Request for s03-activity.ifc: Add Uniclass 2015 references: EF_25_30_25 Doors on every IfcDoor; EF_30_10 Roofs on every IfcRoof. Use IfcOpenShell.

First a look at what the model holds.

```python
import ifcopenshell

model = ifcopenshell.open("s03-activity.ifc")
print(model.schema)
print("classifications:", [c.Name for c in model.by_type("IfcClassification")])
for ifc_class in ("IfcDoor", "IfcRoof", "IfcStair", "IfcWall", "IfcWindow"):
    print(ifc_class, len(model.by_type(ifc_class)))
```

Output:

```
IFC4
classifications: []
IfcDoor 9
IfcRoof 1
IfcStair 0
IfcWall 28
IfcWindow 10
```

```python
import ifcopenshell
import ifcopenshell.api.classification

model = ifcopenshell.open("s03-activity.ifc")

system = ifcopenshell.api.classification.add_classification(model, classification="Uniclass 2015")

codes = {
    "IfcDoor": ("EF_25_30_25", "Doors"),
    "IfcRoof": ("EF_30_10", "Roofs"),
}
for ifc_class, (code, name) in codes.items():
    products = model.by_type(ifc_class)
    ifcopenshell.api.classification.add_reference(
        model, products=products, classification=system, identification=code, name=name
    )
    print(code, len(products))

model.write("s03-activity_rev.ifc")
```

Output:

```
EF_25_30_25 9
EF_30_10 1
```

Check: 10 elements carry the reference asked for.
